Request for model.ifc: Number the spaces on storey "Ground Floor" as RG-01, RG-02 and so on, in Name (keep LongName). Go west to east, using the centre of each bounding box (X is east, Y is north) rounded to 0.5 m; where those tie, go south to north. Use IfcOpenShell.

First a look at what the model holds.

```python
import ifcopenshell
import ifcopenshell.util.element
import ifcopenshell.util.placement

model = ifcopenshell.open("model.ifc")
print(model.schema)
storey = next(s for s in model.by_type("IfcBuildingStorey") if s.Name == "Ground Floor")
spaces = [e for e in ifcopenshell.util.element.get_decomposition(storey) if e.is_a("IfcSpace")]
for e in sorted(spaces, key=lambda e: e.id()):
    origin = ifcopenshell.util.placement.get_local_placement(e.ObjectPlacement)[:3, 3]
    print(e.id(), e.Name, e.LongName, origin.round(2) + 0.0, sep=" | ")
```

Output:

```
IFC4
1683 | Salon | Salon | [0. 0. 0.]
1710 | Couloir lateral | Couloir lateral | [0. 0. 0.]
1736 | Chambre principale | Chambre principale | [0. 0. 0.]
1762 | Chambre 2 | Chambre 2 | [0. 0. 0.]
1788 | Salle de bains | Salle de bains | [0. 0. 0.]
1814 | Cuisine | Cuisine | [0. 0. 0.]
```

```python
import ifcopenshell
import ifcopenshell.geom
import ifcopenshell.util.element
import ifcopenshell.util.shape

model = ifcopenshell.open("model.ifc")
settings = ifcopenshell.geom.settings()
settings.set("use-world-coords", True)


def centre(element):
    shape = ifcopenshell.geom.create_shape(settings, element)
    return ifcopenshell.util.shape.get_bbox_centroid(shape.geometry)


storey = next(s for s in model.by_type("IfcBuildingStorey") if s.Name == "Ground Floor")
spaces = [e for e in ifcopenshell.util.element.get_decomposition(storey) if e.is_a("IfcSpace")]

# Insertion points can sit at a corner or the storey origin, so sort by the geometry (in metres).
centres = {e: centre(e) for e in spaces}
spaces.sort(key=lambda e: (round(centres[e][0] / 0.5), centres[e][1]))

for i, e in enumerate(spaces, start=1):
    number = f"RG-{i:02d}"
    e.Name = number
    print(e.id(), number)

model.write("model_rev.ifc")
```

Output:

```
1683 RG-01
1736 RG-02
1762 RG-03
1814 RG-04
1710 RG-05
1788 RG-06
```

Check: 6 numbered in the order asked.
